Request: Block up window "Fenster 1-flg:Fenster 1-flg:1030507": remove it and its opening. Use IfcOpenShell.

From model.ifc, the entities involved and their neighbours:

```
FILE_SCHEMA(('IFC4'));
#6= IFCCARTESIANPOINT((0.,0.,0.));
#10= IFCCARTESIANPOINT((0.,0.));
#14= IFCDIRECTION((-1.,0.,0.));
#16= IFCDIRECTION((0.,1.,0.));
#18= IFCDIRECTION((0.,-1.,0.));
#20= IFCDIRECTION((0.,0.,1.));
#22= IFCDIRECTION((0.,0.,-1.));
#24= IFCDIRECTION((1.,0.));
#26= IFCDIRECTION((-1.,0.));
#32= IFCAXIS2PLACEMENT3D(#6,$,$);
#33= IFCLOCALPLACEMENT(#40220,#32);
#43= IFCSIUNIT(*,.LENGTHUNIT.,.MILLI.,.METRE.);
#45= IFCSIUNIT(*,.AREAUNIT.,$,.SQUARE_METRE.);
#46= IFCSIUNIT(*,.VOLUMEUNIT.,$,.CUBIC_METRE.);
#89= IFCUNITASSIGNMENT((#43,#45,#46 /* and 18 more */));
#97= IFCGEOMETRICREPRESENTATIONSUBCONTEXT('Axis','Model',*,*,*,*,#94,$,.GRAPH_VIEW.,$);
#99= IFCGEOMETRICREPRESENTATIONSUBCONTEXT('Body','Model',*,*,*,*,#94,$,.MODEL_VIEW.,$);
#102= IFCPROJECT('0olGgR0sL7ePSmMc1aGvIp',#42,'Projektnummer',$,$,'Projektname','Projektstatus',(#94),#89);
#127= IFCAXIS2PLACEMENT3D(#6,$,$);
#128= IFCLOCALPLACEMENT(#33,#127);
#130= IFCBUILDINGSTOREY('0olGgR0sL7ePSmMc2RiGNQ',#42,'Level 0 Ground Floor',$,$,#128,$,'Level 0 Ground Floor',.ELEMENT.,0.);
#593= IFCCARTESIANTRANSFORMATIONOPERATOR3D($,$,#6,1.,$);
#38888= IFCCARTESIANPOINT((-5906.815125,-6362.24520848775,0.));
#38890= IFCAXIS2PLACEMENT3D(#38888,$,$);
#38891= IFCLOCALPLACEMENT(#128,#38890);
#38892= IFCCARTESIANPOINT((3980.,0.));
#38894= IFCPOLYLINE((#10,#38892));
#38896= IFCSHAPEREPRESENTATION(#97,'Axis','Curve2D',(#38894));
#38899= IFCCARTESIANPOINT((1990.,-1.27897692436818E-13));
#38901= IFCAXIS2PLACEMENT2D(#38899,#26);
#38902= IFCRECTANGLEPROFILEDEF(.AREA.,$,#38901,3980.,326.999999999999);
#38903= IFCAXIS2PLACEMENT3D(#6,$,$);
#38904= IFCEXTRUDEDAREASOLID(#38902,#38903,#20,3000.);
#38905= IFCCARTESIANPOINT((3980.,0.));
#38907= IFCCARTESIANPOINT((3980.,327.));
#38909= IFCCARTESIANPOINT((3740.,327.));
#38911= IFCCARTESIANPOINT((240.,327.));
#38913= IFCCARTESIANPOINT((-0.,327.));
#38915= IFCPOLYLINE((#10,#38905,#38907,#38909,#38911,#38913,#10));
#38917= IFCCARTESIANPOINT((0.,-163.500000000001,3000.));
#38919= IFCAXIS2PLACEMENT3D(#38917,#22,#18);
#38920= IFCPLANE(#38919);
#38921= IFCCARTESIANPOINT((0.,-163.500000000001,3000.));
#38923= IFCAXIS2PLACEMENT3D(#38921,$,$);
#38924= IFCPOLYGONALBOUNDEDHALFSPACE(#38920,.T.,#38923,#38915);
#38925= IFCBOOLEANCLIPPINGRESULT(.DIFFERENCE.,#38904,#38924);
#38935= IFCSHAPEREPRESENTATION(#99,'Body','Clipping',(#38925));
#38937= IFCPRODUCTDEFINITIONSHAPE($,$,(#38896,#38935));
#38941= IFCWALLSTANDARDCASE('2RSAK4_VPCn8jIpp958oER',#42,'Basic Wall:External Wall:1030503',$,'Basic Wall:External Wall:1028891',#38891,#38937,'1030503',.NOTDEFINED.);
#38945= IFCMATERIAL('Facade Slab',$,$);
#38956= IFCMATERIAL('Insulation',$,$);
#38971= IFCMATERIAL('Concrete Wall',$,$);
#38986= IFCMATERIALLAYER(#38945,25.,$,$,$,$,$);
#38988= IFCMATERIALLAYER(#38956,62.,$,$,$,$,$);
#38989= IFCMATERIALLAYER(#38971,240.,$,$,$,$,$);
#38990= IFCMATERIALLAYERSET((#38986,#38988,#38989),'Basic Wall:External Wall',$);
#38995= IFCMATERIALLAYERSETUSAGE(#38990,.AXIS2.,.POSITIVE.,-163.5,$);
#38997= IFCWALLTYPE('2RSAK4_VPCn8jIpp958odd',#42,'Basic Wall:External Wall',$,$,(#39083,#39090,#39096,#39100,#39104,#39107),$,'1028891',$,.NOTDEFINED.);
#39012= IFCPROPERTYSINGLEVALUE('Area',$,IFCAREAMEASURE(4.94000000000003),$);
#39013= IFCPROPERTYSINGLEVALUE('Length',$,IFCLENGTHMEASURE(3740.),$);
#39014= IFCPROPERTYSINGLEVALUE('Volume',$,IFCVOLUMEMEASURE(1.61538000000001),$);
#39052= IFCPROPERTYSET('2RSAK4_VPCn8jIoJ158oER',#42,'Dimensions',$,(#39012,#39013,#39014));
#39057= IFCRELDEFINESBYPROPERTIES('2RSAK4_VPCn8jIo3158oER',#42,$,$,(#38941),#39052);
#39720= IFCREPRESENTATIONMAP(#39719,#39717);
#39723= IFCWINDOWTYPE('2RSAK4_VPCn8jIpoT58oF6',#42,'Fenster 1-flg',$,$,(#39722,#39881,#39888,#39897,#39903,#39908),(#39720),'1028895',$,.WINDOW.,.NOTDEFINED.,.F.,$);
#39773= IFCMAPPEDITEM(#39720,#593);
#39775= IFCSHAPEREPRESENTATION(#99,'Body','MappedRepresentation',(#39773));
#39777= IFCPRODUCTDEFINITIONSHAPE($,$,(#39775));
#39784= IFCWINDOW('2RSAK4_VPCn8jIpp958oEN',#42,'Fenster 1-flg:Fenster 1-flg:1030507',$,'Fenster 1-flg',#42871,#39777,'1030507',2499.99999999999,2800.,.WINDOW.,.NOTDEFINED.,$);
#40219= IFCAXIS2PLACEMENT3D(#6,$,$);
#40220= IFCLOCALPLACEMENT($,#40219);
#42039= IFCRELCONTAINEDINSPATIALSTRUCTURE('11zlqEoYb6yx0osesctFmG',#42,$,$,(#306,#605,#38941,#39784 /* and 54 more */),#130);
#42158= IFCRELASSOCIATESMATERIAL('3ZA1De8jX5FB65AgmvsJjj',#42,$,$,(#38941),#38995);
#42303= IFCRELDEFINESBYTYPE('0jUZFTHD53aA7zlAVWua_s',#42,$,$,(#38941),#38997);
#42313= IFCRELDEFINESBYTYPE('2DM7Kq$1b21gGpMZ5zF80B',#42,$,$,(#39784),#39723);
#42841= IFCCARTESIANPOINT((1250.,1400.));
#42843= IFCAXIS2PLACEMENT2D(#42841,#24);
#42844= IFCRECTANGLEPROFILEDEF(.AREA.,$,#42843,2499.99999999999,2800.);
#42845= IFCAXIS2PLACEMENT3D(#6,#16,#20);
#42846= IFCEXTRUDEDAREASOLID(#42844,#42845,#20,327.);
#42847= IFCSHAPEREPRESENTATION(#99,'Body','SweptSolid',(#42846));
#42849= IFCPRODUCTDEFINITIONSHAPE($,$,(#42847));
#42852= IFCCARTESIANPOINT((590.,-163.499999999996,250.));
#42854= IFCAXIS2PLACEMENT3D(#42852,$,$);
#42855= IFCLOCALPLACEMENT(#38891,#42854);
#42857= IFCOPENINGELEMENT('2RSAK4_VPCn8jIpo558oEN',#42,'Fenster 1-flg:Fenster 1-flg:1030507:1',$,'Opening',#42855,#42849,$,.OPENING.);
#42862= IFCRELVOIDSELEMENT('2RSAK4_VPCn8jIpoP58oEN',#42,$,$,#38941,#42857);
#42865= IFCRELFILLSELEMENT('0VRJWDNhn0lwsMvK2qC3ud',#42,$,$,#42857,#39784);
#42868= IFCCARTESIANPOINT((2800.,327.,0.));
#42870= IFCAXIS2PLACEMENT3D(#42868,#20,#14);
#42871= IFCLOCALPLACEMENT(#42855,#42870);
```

```python
import ifcopenshell
import ifcopenshell.api.feature
import ifcopenshell.api.pset
import ifcopenshell.api.root
import ifcopenshell.geom
import ifcopenshell.util.element
import ifcopenshell.util.shape
import ifcopenshell.util.unit

model = ifcopenshell.open("model.ifc")
area_scale = ifcopenshell.util.unit.calculate_unit_scale(model, "AREAUNIT")
volume_scale = ifcopenshell.util.unit.calculate_unit_scale(model, "VOLUMEUNIT")
settings = ifcopenshell.geom.settings()


def volume(element):
    """Net volume in cubic metres, openings subtracted."""
    shape = ifcopenshell.geom.create_shape(settings, element)
    return ifcopenshell.util.shape.get_volume(shape.geometry)


window = model.by_guid("2RSAK4_VPCn8jIpp958oEN")
opening = window.FillsVoids[0].RelatingOpeningElement
wall = opening.VoidsElements[0].RelatingBuildingElement
before = volume(wall)

ifcopenshell.api.root.remove_product(model, product=window)
ifcopenshell.api.feature.remove_feature(model, feature=opening)

after = volume(wall)
thickness = 0.327  # wall thickness in metres

# Update the wall's stored quantities.
pset = model.by_id(ifcopenshell.util.element.get_pset(wall, "Dimensions", should_inherit=False)["id"])
ifcopenshell.api.pset.edit_pset(model, pset=pset, properties={
    "Area": model.create_entity("IfcAreaMeasure", after / thickness / area_scale),
    "Volume": model.create_entity("IfcVolumeMeasure", after / volume_scale),
})

print(f"wall volume {before:.3f} -> {after:.3f} m3")

model.write("model-out.ifc")
```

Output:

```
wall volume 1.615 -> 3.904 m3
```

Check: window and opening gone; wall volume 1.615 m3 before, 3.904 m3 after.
